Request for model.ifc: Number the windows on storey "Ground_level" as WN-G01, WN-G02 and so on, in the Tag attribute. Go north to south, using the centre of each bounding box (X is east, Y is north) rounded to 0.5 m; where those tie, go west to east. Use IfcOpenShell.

First a look at what the model holds.

```python
import ifcopenshell
import ifcopenshell.util.element
import ifcopenshell.util.placement

model = ifcopenshell.open("model.ifc")
print(model.schema)
storey = next(s for s in model.by_type("IfcBuildingStorey") if s.Name == "Ground_level")
windows = [e for e in ifcopenshell.util.element.get_decomposition(storey) if e.is_a("IfcWindow")]
for e in sorted(windows, key=lambda e: e.id()):
    origin = ifcopenshell.util.placement.get_local_placement(e.ObjectPlacement)[:3, 3]
    print(e.id(), e.Tag, e.Name, origin.round(2) + 0.0, sep=" | ")
```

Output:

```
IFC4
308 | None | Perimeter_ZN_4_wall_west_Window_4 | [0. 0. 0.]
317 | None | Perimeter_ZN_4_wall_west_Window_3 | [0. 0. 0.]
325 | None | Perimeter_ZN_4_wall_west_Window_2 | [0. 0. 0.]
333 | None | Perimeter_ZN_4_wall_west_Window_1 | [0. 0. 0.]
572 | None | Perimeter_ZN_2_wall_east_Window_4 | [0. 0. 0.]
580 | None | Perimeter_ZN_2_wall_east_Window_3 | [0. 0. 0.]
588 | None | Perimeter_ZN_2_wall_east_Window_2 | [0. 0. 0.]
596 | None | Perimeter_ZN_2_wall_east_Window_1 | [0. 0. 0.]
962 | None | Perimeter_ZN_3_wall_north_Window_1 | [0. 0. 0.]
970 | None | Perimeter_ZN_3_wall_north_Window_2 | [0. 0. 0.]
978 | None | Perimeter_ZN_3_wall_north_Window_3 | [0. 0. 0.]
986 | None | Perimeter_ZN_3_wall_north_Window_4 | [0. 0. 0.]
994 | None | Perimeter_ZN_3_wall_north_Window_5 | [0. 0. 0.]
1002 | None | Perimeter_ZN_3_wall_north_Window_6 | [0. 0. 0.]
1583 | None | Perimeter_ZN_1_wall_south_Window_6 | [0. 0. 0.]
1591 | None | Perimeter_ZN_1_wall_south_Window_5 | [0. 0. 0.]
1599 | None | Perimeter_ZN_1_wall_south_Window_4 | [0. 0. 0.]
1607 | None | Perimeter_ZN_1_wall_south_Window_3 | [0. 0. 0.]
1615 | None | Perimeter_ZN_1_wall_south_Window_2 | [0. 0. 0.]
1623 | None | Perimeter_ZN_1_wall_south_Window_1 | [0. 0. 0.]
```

```python
import ifcopenshell
import ifcopenshell.geom
import ifcopenshell.util.element
import ifcopenshell.util.shape

model = ifcopenshell.open("model.ifc")
settings = ifcopenshell.geom.settings()
settings.set("use-world-coords", True)


def centre(element):
    shape = ifcopenshell.geom.create_shape(settings, element)
    return ifcopenshell.util.shape.get_bbox_centroid(shape.geometry)


storey = next(s for s in model.by_type("IfcBuildingStorey") if s.Name == "Ground_level")
windows = [e for e in ifcopenshell.util.element.get_decomposition(storey) if e.is_a("IfcWindow")]

# Insertion points can sit at a corner or the storey origin, so sort by the geometry (in metres).
centres = {e: centre(e) for e in windows}
windows.sort(key=lambda e: (-round(centres[e][1] / 0.5), centres[e][0]))

for i, e in enumerate(windows, start=1):
    number = f"WN-G{i:02d}"
    e.Tag = number
    print(e.id(), number)

model.write("model_edited.ifc")
```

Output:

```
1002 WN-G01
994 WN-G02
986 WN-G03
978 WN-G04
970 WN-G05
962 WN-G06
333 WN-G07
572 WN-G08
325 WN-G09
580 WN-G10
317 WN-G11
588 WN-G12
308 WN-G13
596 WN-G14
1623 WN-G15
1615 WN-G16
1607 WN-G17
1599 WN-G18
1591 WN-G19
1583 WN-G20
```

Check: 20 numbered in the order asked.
